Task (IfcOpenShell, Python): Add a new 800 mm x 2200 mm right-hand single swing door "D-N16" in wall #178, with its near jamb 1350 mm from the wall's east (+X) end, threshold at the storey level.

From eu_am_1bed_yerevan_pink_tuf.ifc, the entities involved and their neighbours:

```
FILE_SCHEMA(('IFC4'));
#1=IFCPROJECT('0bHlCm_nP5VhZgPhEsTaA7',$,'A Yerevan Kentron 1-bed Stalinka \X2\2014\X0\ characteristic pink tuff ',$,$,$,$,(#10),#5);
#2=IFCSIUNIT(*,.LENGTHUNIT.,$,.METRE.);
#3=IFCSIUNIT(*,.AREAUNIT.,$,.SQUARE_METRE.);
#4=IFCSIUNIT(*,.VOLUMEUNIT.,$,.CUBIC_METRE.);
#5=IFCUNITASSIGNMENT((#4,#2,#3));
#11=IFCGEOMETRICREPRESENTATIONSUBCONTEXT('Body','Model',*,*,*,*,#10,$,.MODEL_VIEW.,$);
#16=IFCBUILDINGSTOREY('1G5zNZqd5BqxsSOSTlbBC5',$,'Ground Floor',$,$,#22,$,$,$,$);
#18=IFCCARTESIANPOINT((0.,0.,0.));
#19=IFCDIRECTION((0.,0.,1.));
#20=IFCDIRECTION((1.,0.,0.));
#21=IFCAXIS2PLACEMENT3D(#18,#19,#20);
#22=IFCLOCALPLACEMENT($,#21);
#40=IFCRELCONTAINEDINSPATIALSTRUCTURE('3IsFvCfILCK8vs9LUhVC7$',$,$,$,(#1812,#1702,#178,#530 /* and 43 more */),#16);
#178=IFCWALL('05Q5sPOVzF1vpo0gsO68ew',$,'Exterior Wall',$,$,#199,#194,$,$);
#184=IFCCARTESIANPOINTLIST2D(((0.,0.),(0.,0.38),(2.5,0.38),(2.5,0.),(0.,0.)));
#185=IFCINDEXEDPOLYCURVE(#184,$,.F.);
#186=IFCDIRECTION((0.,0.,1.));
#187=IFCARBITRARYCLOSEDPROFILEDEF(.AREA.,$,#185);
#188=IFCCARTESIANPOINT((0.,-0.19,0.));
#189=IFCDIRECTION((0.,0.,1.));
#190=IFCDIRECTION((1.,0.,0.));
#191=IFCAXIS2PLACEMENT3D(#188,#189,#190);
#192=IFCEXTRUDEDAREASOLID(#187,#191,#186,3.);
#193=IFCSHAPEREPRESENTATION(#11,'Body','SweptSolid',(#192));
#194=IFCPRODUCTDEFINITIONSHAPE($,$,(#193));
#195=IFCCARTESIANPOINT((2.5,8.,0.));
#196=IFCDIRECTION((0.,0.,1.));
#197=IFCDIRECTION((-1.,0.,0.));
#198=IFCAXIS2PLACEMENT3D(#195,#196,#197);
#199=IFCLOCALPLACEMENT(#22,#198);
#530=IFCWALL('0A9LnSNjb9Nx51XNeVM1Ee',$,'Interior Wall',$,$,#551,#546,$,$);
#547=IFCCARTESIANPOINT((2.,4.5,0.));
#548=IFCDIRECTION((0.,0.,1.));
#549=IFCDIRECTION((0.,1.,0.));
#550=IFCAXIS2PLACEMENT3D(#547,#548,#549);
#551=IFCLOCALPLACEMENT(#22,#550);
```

```python
import numpy as np
import ifcopenshell
import ifcopenshell.api.feature
import ifcopenshell.api.geometry
import ifcopenshell.api.root
import ifcopenshell.api.spatial
import ifcopenshell.geom
import ifcopenshell.util.element
import ifcopenshell.util.placement
import ifcopenshell.util.representation
import ifcopenshell.util.shape
import ifcopenshell.util.unit

model = ifcopenshell.open("eu_am_1bed_yerevan_pink_tuf.ifc")
unit_scale = ifcopenshell.util.unit.calculate_unit_scale(model)
settings = ifcopenshell.geom.settings()


def volume(element):
    """Net volume in cubic metres, openings subtracted."""
    shape = ifcopenshell.geom.create_shape(settings, element)
    return ifcopenshell.util.shape.get_volume(shape.geometry)


wall = model.by_guid("05Q5sPOVzF1vpo0gsO68ew")
storey = ifcopenshell.util.element.get_container(wall, ifc_class="IfcBuildingStorey")
context = ifcopenshell.util.representation.get_context(model, "Model", "Body", "MODEL_VIEW")
before = volume(wall)

width, height, from_end, sill = 0.8, 2.2, 1.35, 0.0  # metres

# The wall runs along its own X axis, and the end named is its -X end.
wall_shape = ifcopenshell.geom.create_shape(settings, wall)
x, y, z = ifcopenshell.util.shape.get_vertices(wall_shape.geometry).T
start = x.min() + from_end
face, thickness = float(y.min()), float(y.max() - y.min())
wall_matrix = ifcopenshell.util.placement.get_local_placement(wall.ObjectPlacement)
level = ifcopenshell.util.placement.get_local_placement(storey.ObjectPlacement)[2, 3]


def in_wall(x, y):
    """Placement at x, y metres in the wall's axes, at sill height."""
    matrix = wall_matrix.copy()
    matrix[:, 3] = wall_matrix @ np.array([x / unit_scale, y / unit_scale, 0.0, 1.0])
    matrix[2, 3] = level + sill / unit_scale
    return matrix


# Opening: a box that overshoots both wall faces by 50 mm.
opening = ifcopenshell.api.root.create_entity(model, ifc_class="IfcOpeningElement", predefined_type="OPENING")
box = ifcopenshell.api.geometry.add_wall_representation(
    model, context=context, length=width, height=height, thickness=thickness + 0.1
)
ifcopenshell.api.geometry.assign_representation(model, product=opening, representation=box)
ifcopenshell.api.geometry.edit_object_placement(model, product=opening, matrix=in_wall(start, face - 0.05), is_si=False)
ifcopenshell.api.feature.add_feature(model, feature=opening, element=wall)

door = ifcopenshell.api.root.create_entity(model, ifc_class="IfcDoor", name="D-N16", predefined_type="DOOR")
door.OverallWidth, door.OverallHeight = width / unit_scale, height / unit_scale
door.OperationType = "SINGLE_SWING_RIGHT"
body = ifcopenshell.api.geometry.add_door_representation(
    model,
    context=context,
    overall_width=door.OverallWidth,
    overall_height=door.OverallHeight,
    operation_type="SINGLE_SWING_RIGHT",
    lining_properties={"LiningDepth": thickness / unit_scale, "ThresholdDepth": thickness / unit_scale},
)
ifcopenshell.api.geometry.assign_representation(model, product=door, representation=body)
ifcopenshell.api.spatial.assign_container(model, products=[door], relating_structure=storey)
ifcopenshell.api.feature.add_filling(model, opening=opening, element=door)

# The lining spans the wall, so the door starts at the wall face.
ifcopenshell.api.geometry.edit_object_placement(model, product=door, matrix=in_wall(start, face), is_si=False)

after = volume(wall)

print(f"wall volume {before:.3f} -> {after:.3f} m3")

model.write("eu_am_1bed_yerevan_pink_tuf_edited.ifc")
```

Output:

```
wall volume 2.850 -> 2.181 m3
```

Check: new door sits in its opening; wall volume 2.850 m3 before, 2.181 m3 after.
